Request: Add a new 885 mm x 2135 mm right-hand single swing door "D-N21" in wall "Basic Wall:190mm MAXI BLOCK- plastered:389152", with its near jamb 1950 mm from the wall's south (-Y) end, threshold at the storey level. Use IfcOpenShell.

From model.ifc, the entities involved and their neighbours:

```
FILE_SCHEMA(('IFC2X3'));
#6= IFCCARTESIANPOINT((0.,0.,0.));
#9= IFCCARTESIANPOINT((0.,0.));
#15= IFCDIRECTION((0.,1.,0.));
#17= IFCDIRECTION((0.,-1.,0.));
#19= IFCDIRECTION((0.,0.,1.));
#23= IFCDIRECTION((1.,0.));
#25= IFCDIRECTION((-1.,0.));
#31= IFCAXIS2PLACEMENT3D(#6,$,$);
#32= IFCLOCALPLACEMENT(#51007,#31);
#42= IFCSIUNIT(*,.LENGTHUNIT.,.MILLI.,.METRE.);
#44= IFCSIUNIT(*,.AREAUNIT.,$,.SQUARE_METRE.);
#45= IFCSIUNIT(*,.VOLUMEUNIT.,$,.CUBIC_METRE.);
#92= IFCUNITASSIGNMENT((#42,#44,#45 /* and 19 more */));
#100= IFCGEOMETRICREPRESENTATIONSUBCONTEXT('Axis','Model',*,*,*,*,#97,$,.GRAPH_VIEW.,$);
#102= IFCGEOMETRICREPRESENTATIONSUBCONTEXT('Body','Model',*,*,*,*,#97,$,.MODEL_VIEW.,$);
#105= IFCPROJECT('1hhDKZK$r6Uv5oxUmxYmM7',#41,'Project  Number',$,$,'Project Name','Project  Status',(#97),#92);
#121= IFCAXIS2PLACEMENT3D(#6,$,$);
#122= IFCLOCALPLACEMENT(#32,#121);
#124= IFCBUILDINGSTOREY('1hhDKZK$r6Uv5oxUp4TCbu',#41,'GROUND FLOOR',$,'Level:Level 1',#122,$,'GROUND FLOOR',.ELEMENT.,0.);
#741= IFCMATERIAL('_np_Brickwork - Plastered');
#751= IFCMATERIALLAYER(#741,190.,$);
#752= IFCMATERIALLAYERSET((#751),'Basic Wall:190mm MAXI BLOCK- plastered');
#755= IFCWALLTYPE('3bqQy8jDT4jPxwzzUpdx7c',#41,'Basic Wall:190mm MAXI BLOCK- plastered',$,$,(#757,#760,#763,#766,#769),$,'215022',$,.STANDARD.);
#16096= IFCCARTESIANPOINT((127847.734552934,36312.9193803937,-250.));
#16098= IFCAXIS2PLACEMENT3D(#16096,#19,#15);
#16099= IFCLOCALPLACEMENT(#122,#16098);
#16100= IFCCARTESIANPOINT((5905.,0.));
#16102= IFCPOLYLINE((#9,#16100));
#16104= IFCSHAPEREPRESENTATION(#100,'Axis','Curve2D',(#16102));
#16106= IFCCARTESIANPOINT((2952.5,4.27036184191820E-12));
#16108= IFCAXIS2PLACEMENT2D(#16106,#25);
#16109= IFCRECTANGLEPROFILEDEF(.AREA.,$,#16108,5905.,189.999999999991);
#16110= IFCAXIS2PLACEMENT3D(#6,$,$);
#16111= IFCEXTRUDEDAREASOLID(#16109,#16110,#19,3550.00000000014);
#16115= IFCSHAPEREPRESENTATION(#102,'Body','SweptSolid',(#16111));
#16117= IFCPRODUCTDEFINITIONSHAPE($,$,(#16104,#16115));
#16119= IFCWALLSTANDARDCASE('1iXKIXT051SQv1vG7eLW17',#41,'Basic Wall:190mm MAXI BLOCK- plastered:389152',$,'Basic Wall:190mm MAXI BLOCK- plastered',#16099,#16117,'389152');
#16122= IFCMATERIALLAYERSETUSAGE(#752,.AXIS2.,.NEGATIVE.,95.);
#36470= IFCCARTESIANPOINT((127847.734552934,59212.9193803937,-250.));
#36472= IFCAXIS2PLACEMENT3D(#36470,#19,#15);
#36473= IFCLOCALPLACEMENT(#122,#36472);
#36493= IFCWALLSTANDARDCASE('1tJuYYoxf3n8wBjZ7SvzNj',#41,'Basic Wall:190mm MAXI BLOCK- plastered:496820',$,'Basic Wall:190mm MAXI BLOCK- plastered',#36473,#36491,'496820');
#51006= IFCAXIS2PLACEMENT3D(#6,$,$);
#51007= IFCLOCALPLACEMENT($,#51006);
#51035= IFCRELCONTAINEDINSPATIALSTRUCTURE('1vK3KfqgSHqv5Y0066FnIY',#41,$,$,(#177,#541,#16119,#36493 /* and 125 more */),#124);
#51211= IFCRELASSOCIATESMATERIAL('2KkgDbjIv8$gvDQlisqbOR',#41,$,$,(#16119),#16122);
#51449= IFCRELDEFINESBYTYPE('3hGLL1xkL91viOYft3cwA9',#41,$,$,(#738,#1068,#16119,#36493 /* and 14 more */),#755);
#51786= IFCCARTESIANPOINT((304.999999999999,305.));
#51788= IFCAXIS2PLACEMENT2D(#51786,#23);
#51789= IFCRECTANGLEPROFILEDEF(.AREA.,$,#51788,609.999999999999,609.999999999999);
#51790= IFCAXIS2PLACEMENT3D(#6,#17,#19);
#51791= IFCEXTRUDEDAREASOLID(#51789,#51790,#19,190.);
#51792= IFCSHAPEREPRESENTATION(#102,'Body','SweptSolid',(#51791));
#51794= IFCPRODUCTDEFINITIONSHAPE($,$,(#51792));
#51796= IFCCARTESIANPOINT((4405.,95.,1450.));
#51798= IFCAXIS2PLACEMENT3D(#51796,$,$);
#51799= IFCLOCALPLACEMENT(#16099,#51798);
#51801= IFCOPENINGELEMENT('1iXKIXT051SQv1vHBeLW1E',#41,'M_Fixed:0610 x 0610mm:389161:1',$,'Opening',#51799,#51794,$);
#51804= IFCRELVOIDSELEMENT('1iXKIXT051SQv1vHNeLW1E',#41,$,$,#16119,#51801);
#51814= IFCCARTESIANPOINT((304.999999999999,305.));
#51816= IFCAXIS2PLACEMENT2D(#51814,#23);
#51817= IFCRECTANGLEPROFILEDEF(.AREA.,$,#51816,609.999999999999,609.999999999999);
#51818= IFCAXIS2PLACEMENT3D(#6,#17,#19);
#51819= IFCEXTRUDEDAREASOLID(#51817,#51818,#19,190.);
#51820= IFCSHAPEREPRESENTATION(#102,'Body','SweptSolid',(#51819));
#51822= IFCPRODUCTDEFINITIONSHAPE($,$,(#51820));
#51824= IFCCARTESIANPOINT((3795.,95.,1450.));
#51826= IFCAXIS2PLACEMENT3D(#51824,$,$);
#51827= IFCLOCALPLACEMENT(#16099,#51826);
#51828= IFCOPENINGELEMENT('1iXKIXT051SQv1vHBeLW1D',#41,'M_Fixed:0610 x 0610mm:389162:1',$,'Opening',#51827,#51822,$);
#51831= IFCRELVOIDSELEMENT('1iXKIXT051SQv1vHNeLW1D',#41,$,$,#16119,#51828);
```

```python
import numpy as np
import ifcopenshell
import ifcopenshell.api.feature
import ifcopenshell.api.geometry
import ifcopenshell.api.root
import ifcopenshell.api.spatial
import ifcopenshell.api.type
import ifcopenshell.geom
import ifcopenshell.util.element
import ifcopenshell.util.placement
import ifcopenshell.util.representation
import ifcopenshell.util.shape
import ifcopenshell.util.unit

model = ifcopenshell.open("model.ifc")
unit_scale = ifcopenshell.util.unit.calculate_unit_scale(model)
settings = ifcopenshell.geom.settings()


def volume(element):
    """Net volume in cubic metres, openings subtracted."""
    shape = ifcopenshell.geom.create_shape(settings, element)
    return ifcopenshell.util.shape.get_volume(shape.geometry)


wall = model.by_guid("1iXKIXT051SQv1vG7eLW17")
storey = ifcopenshell.util.element.get_container(wall, ifc_class="IfcBuildingStorey")
context = ifcopenshell.util.representation.get_context(model, "Model", "Body", "MODEL_VIEW")
before = volume(wall)

width, height, from_end, sill = 0.885, 2.135, 1.95, 0.0  # metres

# The wall runs along its own X axis, and the end named is its -X end.
wall_shape = ifcopenshell.geom.create_shape(settings, wall)
x, y, z = ifcopenshell.util.shape.get_vertices(wall_shape.geometry).T
start = x.min() + from_end
face, thickness = float(y.min()), float(y.max() - y.min())
wall_matrix = ifcopenshell.util.placement.get_local_placement(wall.ObjectPlacement)
level = ifcopenshell.util.placement.get_local_placement(storey.ObjectPlacement)[2, 3]


def in_wall(x, y):
    """Placement at x, y metres in the wall's axes, at sill height."""
    matrix = wall_matrix.copy()
    matrix[:, 3] = wall_matrix @ np.array([x / unit_scale, y / unit_scale, 0.0, 1.0])
    matrix[2, 3] = level + sill / unit_scale
    return matrix


# Opening: a box that overshoots both wall faces by 50 mm.
opening = ifcopenshell.api.root.create_entity(model, ifc_class="IfcOpeningElement")
box = ifcopenshell.api.geometry.add_wall_representation(
    model, context=context, length=width, height=height, thickness=thickness + 0.1
)
ifcopenshell.api.geometry.assign_representation(model, product=opening, representation=box)
ifcopenshell.api.geometry.edit_object_placement(model, product=opening, matrix=in_wall(start, face - 0.05), is_si=False)
ifcopenshell.api.feature.add_feature(model, feature=opening, element=wall)

door = ifcopenshell.api.root.create_entity(model, ifc_class="IfcDoor", name="D-N21")
door.OverallWidth, door.OverallHeight = width / unit_scale, height / unit_scale
body = ifcopenshell.api.geometry.add_door_representation(
    model,
    context=context,
    overall_width=door.OverallWidth,
    overall_height=door.OverallHeight,
    operation_type="SINGLE_SWING_RIGHT",
    lining_properties={"LiningDepth": thickness / unit_scale, "ThresholdDepth": thickness / unit_scale},
)
ifcopenshell.api.geometry.assign_representation(model, product=door, representation=body)
ifcopenshell.api.spatial.assign_container(model, products=[door], relating_structure=storey)
fills = ifcopenshell.api.feature.add_filling(model, opening=opening, element=door)
fills.OwnerHistory = door.OwnerHistory  # required in IFC2X3

# IFC2X3 keeps the operation on the door style.
style = ifcopenshell.api.root.create_entity(model, ifc_class="IfcDoorStyle", name="D-N21")
style.OperationType, style.ConstructionType = "SINGLE_SWING_RIGHT", "NOTDEFINED"
style.ParameterTakesPrecedence = style.Sizeable = False
ifcopenshell.api.type.assign_type(model, related_objects=[door], relating_type=style)

# The lining spans the wall, so the door starts at the wall face.
ifcopenshell.api.geometry.edit_object_placement(model, product=door, matrix=in_wall(start, face), is_si=False)

after = volume(wall)

print(f"wall volume {before:.3f} -> {after:.3f} m3")

model.write("model_edited.ifc")
```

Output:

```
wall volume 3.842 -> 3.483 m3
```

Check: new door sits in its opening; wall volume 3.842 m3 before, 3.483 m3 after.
